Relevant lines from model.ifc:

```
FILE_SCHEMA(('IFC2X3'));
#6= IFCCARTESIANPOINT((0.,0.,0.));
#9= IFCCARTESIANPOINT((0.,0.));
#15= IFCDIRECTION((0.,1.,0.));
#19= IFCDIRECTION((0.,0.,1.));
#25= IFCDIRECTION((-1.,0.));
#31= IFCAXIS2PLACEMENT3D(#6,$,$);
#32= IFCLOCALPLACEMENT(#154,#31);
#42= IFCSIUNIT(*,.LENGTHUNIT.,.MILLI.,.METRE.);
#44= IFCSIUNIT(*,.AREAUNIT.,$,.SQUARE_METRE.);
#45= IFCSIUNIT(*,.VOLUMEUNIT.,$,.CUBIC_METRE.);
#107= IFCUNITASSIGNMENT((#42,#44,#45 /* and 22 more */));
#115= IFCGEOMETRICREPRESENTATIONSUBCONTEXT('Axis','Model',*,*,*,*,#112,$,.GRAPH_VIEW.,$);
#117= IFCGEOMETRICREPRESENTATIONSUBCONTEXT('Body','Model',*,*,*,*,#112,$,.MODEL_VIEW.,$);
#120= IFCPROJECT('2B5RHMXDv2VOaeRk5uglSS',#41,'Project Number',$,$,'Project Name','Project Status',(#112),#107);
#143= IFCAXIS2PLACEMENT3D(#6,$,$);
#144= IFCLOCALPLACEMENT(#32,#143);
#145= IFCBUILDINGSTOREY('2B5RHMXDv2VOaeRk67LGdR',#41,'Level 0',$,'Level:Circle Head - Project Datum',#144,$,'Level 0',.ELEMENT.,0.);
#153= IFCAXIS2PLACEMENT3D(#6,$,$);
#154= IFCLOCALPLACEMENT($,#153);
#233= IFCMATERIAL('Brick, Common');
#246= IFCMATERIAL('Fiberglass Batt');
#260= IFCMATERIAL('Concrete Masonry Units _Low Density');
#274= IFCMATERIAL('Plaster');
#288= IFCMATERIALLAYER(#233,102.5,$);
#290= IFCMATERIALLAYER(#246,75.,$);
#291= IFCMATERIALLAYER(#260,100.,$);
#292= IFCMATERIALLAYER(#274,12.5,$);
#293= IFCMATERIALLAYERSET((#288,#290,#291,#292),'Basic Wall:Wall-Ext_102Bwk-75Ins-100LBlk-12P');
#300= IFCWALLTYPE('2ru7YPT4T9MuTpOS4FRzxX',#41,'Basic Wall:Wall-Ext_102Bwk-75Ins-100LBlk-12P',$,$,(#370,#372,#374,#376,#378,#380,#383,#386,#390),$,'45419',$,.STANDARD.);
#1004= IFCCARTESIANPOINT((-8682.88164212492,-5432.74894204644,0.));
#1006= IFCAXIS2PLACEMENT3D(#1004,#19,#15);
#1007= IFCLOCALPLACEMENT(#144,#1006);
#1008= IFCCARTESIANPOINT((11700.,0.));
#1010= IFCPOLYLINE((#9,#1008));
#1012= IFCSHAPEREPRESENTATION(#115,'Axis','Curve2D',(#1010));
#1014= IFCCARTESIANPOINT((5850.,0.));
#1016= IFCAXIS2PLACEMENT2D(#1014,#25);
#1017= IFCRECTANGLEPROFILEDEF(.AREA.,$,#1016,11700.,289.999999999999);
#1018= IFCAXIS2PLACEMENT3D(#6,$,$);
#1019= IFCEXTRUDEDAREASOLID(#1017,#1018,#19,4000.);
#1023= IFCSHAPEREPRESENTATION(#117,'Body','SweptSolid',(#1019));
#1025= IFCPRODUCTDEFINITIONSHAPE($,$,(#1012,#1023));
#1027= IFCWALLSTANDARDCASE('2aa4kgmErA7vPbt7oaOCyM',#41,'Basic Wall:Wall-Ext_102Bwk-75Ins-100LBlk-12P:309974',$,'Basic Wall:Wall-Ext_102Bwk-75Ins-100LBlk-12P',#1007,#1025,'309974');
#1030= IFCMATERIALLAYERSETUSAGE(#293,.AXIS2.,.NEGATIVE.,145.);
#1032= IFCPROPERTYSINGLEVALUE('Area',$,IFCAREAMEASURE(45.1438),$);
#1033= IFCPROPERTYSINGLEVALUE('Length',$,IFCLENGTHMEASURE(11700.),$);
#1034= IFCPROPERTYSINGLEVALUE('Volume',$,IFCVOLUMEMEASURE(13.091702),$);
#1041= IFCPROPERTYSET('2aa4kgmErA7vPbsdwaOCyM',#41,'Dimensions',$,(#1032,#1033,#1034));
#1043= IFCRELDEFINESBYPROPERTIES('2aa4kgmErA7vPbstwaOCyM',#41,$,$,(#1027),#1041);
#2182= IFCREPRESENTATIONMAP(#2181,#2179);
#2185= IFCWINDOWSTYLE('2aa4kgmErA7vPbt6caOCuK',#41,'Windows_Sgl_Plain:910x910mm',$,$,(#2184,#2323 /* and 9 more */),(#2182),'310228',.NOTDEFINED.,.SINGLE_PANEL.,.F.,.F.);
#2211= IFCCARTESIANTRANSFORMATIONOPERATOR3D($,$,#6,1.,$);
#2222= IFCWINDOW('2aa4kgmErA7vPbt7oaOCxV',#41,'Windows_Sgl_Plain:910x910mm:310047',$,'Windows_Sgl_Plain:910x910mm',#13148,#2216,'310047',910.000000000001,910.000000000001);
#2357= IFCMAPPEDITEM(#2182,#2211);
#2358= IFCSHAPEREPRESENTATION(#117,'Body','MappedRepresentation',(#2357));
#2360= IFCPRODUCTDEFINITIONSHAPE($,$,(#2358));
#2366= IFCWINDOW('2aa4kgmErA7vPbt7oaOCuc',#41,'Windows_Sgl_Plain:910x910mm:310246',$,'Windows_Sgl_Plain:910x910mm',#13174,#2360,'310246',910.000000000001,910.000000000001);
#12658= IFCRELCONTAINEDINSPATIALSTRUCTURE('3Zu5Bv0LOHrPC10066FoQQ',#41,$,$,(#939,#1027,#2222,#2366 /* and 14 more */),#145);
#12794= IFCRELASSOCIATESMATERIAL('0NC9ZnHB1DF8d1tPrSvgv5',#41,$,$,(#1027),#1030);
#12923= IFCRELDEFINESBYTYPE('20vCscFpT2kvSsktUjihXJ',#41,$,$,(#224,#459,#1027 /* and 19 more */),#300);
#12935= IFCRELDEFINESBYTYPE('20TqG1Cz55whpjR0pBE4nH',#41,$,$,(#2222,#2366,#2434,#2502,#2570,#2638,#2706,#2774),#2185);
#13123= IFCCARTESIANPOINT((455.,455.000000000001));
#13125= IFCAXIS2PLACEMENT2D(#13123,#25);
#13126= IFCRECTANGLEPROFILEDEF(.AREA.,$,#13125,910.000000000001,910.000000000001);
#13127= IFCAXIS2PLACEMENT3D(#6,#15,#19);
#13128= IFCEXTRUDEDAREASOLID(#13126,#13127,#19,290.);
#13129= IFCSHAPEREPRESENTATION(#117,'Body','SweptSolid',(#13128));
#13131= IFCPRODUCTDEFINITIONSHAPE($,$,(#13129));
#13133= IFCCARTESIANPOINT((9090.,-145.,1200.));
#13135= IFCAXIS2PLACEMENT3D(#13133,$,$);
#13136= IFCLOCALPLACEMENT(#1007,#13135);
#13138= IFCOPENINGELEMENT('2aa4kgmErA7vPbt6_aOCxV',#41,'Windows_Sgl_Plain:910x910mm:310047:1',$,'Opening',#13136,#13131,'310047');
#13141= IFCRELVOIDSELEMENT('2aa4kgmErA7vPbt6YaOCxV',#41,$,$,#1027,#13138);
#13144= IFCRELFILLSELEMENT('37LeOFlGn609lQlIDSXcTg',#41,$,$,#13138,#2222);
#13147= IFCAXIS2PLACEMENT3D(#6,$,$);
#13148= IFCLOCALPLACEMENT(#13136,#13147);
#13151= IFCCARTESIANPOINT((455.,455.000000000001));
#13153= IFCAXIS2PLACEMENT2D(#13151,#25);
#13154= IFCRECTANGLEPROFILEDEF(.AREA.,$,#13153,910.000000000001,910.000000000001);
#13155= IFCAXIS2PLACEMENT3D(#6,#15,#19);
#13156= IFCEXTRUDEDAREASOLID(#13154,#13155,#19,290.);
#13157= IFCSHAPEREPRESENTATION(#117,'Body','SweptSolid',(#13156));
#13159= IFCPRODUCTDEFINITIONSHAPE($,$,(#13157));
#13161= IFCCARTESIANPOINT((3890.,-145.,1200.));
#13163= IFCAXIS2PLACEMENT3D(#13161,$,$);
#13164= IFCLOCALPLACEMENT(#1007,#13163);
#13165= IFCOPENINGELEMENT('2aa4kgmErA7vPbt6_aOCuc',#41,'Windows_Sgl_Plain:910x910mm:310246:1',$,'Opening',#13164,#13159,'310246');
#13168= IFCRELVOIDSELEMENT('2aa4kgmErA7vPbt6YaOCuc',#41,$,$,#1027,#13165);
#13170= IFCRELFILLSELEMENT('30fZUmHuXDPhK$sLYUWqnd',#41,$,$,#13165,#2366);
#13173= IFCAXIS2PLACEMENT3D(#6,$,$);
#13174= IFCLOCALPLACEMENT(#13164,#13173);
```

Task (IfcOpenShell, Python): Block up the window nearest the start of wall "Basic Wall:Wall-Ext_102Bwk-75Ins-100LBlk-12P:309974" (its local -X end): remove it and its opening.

```python
import ifcopenshell
import ifcopenshell.api.feature
import ifcopenshell.api.pset
import ifcopenshell.api.root
import ifcopenshell.geom
import ifcopenshell.util.element
import ifcopenshell.util.shape
import ifcopenshell.util.unit

model = ifcopenshell.open("model.ifc")
area_scale = ifcopenshell.util.unit.calculate_unit_scale(model, "AREAUNIT")
volume_scale = ifcopenshell.util.unit.calculate_unit_scale(model, "VOLUMEUNIT")
settings = ifcopenshell.geom.settings()


def volume(element):
    """Net volume in cubic metres, openings subtracted."""
    shape = ifcopenshell.geom.create_shape(settings, element)
    return ifcopenshell.util.shape.get_volume(shape.geometry)


window = model.by_id(2366)
opening = window.FillsVoids[0].RelatingOpeningElement
wall = opening.VoidsElements[0].RelatingBuildingElement
before = volume(wall)

ifcopenshell.api.root.remove_product(model, product=window)
ifcopenshell.api.feature.remove_feature(model, feature=opening)

after = volume(wall)
thickness = 0.29  # wall thickness in metres

# Update the wall's stored quantities.
pset = model.by_id(ifcopenshell.util.element.get_pset(wall, "Dimensions", should_inherit=False)["id"])
ifcopenshell.api.pset.edit_pset(model, pset=pset, properties={
    "Area": model.create_entity("IfcAreaMeasure", after / thickness / area_scale),
    "Volume": model.create_entity("IfcVolumeMeasure", after / volume_scale),
})

print(f"wall volume {before:.3f} -> {after:.3f} m3")

model.write("model-out.ifc")
```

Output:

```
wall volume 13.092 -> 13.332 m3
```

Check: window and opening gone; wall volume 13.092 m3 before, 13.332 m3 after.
